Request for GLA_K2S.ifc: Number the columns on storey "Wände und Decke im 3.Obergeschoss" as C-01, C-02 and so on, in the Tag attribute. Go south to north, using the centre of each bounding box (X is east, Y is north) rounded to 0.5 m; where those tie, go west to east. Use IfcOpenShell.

First a look at what the model holds.

```python
import ifcopenshell
import ifcopenshell.util.element
import ifcopenshell.util.placement

model = ifcopenshell.open("GLA_K2S.ifc")
print(model.schema)
storey = next(s for s in model.by_type("IfcBuildingStorey") if s.Name == "Wände und Decke im 3.Obergeschoss")
columns = [e for e in ifcopenshell.util.element.get_decomposition(storey) if e.is_a("IfcColumn")]
for e in sorted(columns, key=lambda e: e.id()):
    origin = ifcopenshell.util.placement.get_local_placement(e.ObjectPlacement)[:3, 3]
    print(e.id(), e.Tag, e.Name, origin.round(2) + 0.0, sep=" | ")
```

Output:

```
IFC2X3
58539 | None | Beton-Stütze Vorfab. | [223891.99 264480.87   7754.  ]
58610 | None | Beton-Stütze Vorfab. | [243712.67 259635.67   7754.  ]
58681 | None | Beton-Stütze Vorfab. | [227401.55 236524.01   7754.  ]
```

```python
import ifcopenshell
import ifcopenshell.geom
import ifcopenshell.util.element
import ifcopenshell.util.shape

model = ifcopenshell.open("GLA_K2S.ifc")
settings = ifcopenshell.geom.settings()
settings.set("use-world-coords", True)


def centre(element):
    shape = ifcopenshell.geom.create_shape(settings, element)
    return ifcopenshell.util.shape.get_bbox_centroid(shape.geometry)


storey = next(s for s in model.by_type("IfcBuildingStorey") if s.Name == "Wände und Decke im 3.Obergeschoss")
columns = [e for e in ifcopenshell.util.element.get_decomposition(storey) if e.is_a("IfcColumn")]

# Insertion points can sit at a corner or the storey origin, so sort by the geometry (in metres).
centres = {e: centre(e) for e in columns}
columns.sort(key=lambda e: (round(centres[e][1] / 0.5), centres[e][0]))

for i, e in enumerate(columns, start=1):
    number = f"C-{i:02d}"
    e.Tag = number
    print(e.id(), number)

model.write("GLA_K2S-out.ifc")
```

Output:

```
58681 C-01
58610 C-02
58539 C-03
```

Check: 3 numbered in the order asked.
